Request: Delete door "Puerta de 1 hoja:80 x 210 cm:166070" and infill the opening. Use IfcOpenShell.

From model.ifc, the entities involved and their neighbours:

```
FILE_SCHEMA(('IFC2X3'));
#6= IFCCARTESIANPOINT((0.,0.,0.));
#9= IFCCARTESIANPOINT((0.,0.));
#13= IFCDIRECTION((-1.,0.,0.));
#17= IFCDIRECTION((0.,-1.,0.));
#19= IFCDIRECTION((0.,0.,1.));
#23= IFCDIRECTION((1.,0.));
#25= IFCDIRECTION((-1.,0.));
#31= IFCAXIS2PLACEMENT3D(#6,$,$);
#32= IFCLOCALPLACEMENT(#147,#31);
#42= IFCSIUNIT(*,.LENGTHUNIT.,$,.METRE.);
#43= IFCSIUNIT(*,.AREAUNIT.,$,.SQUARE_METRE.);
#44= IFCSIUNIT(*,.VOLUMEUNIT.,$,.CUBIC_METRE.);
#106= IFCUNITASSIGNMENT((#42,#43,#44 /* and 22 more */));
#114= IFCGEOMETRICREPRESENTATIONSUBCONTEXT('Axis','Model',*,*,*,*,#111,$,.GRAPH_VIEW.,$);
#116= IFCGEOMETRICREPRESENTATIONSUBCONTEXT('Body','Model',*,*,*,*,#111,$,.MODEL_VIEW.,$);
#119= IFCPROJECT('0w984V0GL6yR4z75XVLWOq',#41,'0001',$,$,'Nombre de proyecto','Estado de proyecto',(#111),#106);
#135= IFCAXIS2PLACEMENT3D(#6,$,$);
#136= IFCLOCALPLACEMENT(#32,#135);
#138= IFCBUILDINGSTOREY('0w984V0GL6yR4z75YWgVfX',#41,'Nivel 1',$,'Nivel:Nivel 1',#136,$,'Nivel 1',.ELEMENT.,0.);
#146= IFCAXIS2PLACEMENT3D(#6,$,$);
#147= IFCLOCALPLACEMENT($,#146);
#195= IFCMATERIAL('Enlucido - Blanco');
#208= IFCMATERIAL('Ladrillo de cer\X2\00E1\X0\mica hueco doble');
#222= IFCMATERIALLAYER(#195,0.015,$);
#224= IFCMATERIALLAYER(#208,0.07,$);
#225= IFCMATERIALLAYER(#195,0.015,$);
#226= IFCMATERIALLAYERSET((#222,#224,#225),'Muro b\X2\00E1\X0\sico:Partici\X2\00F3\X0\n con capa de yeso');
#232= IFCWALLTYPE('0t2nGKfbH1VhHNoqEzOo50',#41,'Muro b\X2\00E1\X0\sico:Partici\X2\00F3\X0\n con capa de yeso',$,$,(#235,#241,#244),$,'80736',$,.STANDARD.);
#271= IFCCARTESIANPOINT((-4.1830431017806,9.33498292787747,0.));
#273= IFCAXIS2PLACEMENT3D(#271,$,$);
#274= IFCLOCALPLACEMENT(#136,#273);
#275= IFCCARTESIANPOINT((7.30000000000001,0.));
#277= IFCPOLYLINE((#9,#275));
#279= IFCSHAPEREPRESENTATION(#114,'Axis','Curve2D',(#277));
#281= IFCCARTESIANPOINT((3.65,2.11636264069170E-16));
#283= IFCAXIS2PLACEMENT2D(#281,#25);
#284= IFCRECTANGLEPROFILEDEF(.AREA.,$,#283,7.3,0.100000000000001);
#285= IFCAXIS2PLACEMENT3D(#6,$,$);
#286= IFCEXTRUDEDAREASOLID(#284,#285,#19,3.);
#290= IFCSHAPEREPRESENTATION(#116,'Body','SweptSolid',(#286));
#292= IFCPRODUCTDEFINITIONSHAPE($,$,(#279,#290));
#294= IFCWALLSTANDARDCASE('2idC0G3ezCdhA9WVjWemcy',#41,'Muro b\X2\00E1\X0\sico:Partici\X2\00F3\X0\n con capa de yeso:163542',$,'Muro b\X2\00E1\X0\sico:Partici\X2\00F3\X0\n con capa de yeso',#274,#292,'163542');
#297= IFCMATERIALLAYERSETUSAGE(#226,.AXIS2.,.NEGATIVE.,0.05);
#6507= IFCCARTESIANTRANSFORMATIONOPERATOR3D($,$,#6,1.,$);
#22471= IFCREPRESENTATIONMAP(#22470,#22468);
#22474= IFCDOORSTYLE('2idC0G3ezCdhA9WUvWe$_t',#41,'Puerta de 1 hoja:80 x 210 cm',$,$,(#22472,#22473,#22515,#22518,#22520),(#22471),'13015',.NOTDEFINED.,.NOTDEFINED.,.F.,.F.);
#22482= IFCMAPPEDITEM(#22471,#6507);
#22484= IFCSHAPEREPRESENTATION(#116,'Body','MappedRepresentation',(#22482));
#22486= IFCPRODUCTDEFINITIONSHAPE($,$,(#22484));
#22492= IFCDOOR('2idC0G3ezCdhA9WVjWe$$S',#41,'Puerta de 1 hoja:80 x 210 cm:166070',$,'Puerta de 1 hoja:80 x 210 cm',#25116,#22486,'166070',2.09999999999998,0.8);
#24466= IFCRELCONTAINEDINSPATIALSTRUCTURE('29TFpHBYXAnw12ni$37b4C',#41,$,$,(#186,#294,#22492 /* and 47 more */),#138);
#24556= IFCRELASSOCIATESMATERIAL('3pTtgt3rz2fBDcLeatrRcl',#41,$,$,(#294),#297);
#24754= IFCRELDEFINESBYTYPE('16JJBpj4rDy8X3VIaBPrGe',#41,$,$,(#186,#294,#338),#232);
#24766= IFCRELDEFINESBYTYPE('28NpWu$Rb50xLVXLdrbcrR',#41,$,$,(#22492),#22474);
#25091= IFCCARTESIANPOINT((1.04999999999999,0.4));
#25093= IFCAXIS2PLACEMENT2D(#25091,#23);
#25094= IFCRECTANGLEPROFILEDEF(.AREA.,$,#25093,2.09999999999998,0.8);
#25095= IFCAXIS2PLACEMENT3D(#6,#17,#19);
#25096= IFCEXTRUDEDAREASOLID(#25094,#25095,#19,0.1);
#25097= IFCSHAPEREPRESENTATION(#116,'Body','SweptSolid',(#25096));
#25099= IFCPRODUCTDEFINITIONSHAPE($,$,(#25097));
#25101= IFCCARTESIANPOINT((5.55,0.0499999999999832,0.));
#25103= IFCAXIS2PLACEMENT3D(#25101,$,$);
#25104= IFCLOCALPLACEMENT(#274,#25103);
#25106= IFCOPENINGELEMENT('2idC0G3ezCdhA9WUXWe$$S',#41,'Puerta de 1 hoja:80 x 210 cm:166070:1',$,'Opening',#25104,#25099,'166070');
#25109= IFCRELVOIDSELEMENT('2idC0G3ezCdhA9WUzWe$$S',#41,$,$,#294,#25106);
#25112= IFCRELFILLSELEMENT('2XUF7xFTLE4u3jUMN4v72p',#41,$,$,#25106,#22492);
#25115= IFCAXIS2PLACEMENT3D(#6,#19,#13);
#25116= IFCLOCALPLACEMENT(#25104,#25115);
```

```python
import ifcopenshell
import ifcopenshell.api.feature
import ifcopenshell.api.root
import ifcopenshell.geom
import ifcopenshell.util.shape

model = ifcopenshell.open("model.ifc")
settings = ifcopenshell.geom.settings()


def volume(element):
    """Net volume in cubic metres, openings subtracted."""
    shape = ifcopenshell.geom.create_shape(settings, element)
    return ifcopenshell.util.shape.get_volume(shape.geometry)


door = model.by_guid("2idC0G3ezCdhA9WVjWe$$S")
opening = door.FillsVoids[0].RelatingOpeningElement
wall = opening.VoidsElements[0].RelatingBuildingElement
before = volume(wall)

ifcopenshell.api.root.remove_product(model, product=door)
ifcopenshell.api.feature.remove_feature(model, feature=opening)

after = volume(wall)

print(f"wall volume {before:.3f} -> {after:.3f} m3")

model.write("model_v2.ifc")
```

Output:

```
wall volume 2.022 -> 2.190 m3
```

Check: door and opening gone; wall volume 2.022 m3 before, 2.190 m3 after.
